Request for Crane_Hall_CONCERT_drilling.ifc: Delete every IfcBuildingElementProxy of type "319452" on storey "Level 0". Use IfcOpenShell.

First a look at what the model holds.

```python
import ifcopenshell
import ifcopenshell.util.element

model = ifcopenshell.open("Crane_Hall_CONCERT_drilling.ifc")
print(model.schema)
storey = next(s for s in model.by_type("IfcBuildingStorey") if s.Name == "Level 0")
proxies = [e for e in ifcopenshell.util.element.get_decomposition(storey) if e.is_a("IfcBuildingElementProxy")]
seen = {}
for e in proxies:
    element_type = ifcopenshell.util.element.get_type(e)
    name = element_type.Name if element_type not in (None, e) else None
    seen[name] = seen.get(name, 0) + 1
for name, count in sorted(seen.items(), key=str):
    print(count, "x", name)
```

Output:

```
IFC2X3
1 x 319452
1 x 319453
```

```python
import ifcopenshell
import ifcopenshell.api.root
import ifcopenshell.util.element

model = ifcopenshell.open("Crane_Hall_CONCERT_drilling.ifc")

storey = next(s for s in model.by_type("IfcBuildingStorey") if s.Name == "Level 0")
proxies = [e for e in ifcopenshell.util.element.get_decomposition(storey) if e.is_a("IfcBuildingElementProxy")]
targets = [e for e in proxies if (t := ifcopenshell.util.element.get_type(e)) not in (None, e) and t.Name == "319452"]

for e in targets:
    ifcopenshell.api.root.remove_product(model, product=e)
print(len(targets), "removed")

model.write("Crane_Hall_CONCERT_drilling_v2.ifc")
```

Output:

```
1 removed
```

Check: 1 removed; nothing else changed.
